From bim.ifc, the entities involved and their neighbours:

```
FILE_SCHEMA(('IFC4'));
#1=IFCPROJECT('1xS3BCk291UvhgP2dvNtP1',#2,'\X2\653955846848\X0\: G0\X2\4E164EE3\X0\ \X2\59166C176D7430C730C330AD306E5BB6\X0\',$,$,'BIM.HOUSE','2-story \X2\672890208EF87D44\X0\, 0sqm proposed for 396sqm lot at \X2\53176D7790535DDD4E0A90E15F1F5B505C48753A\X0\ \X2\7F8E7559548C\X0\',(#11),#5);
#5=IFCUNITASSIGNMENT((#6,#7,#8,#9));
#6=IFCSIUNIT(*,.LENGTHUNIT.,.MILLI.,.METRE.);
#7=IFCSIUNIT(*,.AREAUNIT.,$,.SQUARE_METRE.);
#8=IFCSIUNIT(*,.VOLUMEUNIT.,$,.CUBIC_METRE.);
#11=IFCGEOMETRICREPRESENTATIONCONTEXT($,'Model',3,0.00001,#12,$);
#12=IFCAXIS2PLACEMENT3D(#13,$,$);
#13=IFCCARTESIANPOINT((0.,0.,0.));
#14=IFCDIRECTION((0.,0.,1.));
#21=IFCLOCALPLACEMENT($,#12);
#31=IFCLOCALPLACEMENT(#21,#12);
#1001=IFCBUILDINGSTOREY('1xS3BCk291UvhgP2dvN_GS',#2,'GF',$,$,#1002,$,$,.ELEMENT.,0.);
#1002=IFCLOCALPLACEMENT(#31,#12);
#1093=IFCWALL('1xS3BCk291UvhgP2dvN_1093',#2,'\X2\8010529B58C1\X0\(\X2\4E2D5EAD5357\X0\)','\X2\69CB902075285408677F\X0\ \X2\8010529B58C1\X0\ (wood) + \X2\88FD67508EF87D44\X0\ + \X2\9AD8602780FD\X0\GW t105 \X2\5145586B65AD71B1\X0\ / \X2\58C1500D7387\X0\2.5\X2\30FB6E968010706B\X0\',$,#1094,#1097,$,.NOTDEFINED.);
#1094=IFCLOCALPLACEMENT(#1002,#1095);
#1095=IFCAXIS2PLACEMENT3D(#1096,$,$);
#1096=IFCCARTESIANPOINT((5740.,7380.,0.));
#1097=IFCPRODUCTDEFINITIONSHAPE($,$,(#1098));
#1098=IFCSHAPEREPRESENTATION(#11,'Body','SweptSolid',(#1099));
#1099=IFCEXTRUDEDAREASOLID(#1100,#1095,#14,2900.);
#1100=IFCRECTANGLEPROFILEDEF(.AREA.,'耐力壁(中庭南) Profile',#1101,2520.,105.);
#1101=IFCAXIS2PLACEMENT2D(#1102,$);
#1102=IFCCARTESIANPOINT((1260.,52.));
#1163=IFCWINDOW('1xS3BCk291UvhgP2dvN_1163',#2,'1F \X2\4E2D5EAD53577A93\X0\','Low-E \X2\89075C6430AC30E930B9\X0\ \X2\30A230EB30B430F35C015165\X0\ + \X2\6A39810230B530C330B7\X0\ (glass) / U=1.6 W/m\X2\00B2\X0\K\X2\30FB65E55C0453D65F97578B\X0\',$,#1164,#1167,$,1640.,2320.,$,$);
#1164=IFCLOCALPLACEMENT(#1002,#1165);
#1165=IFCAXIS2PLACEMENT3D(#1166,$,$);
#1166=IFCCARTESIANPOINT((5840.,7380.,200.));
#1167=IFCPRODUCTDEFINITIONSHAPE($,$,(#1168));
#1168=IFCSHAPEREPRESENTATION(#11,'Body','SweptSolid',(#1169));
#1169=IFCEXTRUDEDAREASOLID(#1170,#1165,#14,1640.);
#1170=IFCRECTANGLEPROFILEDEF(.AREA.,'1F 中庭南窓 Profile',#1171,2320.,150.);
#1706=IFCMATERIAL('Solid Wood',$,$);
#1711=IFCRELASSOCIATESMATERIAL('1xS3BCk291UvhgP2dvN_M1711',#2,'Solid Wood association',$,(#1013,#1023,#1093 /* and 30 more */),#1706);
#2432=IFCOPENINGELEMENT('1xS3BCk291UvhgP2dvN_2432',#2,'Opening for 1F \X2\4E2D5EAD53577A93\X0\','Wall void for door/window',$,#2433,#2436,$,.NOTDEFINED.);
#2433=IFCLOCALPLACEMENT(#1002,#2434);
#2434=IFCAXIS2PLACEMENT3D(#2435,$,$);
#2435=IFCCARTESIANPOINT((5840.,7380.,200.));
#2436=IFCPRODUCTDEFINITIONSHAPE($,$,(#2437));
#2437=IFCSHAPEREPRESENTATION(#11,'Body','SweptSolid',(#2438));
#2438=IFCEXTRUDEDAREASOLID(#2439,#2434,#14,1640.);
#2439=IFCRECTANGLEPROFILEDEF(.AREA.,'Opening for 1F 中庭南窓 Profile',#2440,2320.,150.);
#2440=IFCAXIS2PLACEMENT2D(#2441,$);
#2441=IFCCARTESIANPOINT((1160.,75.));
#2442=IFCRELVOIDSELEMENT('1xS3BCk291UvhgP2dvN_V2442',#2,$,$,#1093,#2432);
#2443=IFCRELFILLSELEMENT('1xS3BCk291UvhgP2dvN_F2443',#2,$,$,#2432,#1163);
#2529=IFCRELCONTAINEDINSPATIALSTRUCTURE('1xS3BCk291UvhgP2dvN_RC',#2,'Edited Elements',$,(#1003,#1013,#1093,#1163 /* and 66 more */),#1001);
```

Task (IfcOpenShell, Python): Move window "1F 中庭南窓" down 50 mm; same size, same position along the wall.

```python
import numpy as np
import ifcopenshell
import ifcopenshell.api.geometry
import ifcopenshell.util.placement
import ifcopenshell.util.unit

model = ifcopenshell.open("bim.ifc")
unit_scale = ifcopenshell.util.unit.calculate_unit_scale(model)

window = model.by_guid("1xS3BCk291UvhgP2dvN_1163")
opening = window.FillsVoids[0].RelatingOpeningElement
dz = -0.05 / unit_scale

shift = np.array([0.0, 0.0, dz])
# The window is not placed relative to its opening, so move both.
for product in (opening, window):
    matrix = ifcopenshell.util.placement.get_local_placement(product.ObjectPlacement)
    matrix[:3, 3] += shift
    ifcopenshell.api.geometry.edit_object_placement(model, product=product, matrix=matrix, is_si=False)

print(f"moved by {dz * unit_scale:+.3f} m")

model.write("bim_v2.ifc")
```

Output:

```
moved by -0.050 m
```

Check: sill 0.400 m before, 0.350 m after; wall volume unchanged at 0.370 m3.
